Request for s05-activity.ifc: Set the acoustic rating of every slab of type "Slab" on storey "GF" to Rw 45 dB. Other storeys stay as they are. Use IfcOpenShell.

First a look at what the model holds.

```python
import ifcopenshell
import ifcopenshell.util.element

model = ifcopenshell.open("s05-activity.ifc")
print(model.schema)
storey = next(s for s in model.by_type("IfcBuildingStorey") if s.Name == "GF")
slabs = [e for e in ifcopenshell.util.element.get_decomposition(storey) if e.is_a("IfcSlab")]
seen = {}
for e in slabs:
    element_type = ifcopenshell.util.element.get_type(e)
    key = (element_type.Name if element_type != e and element_type else None, ifcopenshell.util.element.get_pset(e, "Pset_SlabCommon", "AcousticRating"))
    seen[key] = seen.get(key, 0) + 1
for (name, value), count in sorted(seen.items(), key=str):
    print(count, "x", name, "|", value)
```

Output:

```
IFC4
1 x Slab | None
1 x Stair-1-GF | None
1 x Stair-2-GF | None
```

```python
import ifcopenshell
import ifcopenshell.api.pset
import ifcopenshell.util.element

model = ifcopenshell.open("s05-activity.ifc")

storey = next(s for s in model.by_type("IfcBuildingStorey") if s.Name == "GF")
slabs = [e for e in ifcopenshell.util.element.get_decomposition(storey) if e.is_a("IfcSlab")]

count = 0
for e in slabs:
    element_type = ifcopenshell.util.element.get_type(e)
    if element_type in (None, e) or element_type.Name != "Slab":
        continue
    # add_pset returns the element's existing set when there is one.
    pset = ifcopenshell.api.pset.add_pset(model, product=e, name="Pset_SlabCommon")
    ifcopenshell.api.pset.edit_pset(model, pset=pset, properties={"AcousticRating": "Rw 45 dB"})
    count += 1

print(count, "slabs updated")

model.write("s05-activity_edited.ifc")
```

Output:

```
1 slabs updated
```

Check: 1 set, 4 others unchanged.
